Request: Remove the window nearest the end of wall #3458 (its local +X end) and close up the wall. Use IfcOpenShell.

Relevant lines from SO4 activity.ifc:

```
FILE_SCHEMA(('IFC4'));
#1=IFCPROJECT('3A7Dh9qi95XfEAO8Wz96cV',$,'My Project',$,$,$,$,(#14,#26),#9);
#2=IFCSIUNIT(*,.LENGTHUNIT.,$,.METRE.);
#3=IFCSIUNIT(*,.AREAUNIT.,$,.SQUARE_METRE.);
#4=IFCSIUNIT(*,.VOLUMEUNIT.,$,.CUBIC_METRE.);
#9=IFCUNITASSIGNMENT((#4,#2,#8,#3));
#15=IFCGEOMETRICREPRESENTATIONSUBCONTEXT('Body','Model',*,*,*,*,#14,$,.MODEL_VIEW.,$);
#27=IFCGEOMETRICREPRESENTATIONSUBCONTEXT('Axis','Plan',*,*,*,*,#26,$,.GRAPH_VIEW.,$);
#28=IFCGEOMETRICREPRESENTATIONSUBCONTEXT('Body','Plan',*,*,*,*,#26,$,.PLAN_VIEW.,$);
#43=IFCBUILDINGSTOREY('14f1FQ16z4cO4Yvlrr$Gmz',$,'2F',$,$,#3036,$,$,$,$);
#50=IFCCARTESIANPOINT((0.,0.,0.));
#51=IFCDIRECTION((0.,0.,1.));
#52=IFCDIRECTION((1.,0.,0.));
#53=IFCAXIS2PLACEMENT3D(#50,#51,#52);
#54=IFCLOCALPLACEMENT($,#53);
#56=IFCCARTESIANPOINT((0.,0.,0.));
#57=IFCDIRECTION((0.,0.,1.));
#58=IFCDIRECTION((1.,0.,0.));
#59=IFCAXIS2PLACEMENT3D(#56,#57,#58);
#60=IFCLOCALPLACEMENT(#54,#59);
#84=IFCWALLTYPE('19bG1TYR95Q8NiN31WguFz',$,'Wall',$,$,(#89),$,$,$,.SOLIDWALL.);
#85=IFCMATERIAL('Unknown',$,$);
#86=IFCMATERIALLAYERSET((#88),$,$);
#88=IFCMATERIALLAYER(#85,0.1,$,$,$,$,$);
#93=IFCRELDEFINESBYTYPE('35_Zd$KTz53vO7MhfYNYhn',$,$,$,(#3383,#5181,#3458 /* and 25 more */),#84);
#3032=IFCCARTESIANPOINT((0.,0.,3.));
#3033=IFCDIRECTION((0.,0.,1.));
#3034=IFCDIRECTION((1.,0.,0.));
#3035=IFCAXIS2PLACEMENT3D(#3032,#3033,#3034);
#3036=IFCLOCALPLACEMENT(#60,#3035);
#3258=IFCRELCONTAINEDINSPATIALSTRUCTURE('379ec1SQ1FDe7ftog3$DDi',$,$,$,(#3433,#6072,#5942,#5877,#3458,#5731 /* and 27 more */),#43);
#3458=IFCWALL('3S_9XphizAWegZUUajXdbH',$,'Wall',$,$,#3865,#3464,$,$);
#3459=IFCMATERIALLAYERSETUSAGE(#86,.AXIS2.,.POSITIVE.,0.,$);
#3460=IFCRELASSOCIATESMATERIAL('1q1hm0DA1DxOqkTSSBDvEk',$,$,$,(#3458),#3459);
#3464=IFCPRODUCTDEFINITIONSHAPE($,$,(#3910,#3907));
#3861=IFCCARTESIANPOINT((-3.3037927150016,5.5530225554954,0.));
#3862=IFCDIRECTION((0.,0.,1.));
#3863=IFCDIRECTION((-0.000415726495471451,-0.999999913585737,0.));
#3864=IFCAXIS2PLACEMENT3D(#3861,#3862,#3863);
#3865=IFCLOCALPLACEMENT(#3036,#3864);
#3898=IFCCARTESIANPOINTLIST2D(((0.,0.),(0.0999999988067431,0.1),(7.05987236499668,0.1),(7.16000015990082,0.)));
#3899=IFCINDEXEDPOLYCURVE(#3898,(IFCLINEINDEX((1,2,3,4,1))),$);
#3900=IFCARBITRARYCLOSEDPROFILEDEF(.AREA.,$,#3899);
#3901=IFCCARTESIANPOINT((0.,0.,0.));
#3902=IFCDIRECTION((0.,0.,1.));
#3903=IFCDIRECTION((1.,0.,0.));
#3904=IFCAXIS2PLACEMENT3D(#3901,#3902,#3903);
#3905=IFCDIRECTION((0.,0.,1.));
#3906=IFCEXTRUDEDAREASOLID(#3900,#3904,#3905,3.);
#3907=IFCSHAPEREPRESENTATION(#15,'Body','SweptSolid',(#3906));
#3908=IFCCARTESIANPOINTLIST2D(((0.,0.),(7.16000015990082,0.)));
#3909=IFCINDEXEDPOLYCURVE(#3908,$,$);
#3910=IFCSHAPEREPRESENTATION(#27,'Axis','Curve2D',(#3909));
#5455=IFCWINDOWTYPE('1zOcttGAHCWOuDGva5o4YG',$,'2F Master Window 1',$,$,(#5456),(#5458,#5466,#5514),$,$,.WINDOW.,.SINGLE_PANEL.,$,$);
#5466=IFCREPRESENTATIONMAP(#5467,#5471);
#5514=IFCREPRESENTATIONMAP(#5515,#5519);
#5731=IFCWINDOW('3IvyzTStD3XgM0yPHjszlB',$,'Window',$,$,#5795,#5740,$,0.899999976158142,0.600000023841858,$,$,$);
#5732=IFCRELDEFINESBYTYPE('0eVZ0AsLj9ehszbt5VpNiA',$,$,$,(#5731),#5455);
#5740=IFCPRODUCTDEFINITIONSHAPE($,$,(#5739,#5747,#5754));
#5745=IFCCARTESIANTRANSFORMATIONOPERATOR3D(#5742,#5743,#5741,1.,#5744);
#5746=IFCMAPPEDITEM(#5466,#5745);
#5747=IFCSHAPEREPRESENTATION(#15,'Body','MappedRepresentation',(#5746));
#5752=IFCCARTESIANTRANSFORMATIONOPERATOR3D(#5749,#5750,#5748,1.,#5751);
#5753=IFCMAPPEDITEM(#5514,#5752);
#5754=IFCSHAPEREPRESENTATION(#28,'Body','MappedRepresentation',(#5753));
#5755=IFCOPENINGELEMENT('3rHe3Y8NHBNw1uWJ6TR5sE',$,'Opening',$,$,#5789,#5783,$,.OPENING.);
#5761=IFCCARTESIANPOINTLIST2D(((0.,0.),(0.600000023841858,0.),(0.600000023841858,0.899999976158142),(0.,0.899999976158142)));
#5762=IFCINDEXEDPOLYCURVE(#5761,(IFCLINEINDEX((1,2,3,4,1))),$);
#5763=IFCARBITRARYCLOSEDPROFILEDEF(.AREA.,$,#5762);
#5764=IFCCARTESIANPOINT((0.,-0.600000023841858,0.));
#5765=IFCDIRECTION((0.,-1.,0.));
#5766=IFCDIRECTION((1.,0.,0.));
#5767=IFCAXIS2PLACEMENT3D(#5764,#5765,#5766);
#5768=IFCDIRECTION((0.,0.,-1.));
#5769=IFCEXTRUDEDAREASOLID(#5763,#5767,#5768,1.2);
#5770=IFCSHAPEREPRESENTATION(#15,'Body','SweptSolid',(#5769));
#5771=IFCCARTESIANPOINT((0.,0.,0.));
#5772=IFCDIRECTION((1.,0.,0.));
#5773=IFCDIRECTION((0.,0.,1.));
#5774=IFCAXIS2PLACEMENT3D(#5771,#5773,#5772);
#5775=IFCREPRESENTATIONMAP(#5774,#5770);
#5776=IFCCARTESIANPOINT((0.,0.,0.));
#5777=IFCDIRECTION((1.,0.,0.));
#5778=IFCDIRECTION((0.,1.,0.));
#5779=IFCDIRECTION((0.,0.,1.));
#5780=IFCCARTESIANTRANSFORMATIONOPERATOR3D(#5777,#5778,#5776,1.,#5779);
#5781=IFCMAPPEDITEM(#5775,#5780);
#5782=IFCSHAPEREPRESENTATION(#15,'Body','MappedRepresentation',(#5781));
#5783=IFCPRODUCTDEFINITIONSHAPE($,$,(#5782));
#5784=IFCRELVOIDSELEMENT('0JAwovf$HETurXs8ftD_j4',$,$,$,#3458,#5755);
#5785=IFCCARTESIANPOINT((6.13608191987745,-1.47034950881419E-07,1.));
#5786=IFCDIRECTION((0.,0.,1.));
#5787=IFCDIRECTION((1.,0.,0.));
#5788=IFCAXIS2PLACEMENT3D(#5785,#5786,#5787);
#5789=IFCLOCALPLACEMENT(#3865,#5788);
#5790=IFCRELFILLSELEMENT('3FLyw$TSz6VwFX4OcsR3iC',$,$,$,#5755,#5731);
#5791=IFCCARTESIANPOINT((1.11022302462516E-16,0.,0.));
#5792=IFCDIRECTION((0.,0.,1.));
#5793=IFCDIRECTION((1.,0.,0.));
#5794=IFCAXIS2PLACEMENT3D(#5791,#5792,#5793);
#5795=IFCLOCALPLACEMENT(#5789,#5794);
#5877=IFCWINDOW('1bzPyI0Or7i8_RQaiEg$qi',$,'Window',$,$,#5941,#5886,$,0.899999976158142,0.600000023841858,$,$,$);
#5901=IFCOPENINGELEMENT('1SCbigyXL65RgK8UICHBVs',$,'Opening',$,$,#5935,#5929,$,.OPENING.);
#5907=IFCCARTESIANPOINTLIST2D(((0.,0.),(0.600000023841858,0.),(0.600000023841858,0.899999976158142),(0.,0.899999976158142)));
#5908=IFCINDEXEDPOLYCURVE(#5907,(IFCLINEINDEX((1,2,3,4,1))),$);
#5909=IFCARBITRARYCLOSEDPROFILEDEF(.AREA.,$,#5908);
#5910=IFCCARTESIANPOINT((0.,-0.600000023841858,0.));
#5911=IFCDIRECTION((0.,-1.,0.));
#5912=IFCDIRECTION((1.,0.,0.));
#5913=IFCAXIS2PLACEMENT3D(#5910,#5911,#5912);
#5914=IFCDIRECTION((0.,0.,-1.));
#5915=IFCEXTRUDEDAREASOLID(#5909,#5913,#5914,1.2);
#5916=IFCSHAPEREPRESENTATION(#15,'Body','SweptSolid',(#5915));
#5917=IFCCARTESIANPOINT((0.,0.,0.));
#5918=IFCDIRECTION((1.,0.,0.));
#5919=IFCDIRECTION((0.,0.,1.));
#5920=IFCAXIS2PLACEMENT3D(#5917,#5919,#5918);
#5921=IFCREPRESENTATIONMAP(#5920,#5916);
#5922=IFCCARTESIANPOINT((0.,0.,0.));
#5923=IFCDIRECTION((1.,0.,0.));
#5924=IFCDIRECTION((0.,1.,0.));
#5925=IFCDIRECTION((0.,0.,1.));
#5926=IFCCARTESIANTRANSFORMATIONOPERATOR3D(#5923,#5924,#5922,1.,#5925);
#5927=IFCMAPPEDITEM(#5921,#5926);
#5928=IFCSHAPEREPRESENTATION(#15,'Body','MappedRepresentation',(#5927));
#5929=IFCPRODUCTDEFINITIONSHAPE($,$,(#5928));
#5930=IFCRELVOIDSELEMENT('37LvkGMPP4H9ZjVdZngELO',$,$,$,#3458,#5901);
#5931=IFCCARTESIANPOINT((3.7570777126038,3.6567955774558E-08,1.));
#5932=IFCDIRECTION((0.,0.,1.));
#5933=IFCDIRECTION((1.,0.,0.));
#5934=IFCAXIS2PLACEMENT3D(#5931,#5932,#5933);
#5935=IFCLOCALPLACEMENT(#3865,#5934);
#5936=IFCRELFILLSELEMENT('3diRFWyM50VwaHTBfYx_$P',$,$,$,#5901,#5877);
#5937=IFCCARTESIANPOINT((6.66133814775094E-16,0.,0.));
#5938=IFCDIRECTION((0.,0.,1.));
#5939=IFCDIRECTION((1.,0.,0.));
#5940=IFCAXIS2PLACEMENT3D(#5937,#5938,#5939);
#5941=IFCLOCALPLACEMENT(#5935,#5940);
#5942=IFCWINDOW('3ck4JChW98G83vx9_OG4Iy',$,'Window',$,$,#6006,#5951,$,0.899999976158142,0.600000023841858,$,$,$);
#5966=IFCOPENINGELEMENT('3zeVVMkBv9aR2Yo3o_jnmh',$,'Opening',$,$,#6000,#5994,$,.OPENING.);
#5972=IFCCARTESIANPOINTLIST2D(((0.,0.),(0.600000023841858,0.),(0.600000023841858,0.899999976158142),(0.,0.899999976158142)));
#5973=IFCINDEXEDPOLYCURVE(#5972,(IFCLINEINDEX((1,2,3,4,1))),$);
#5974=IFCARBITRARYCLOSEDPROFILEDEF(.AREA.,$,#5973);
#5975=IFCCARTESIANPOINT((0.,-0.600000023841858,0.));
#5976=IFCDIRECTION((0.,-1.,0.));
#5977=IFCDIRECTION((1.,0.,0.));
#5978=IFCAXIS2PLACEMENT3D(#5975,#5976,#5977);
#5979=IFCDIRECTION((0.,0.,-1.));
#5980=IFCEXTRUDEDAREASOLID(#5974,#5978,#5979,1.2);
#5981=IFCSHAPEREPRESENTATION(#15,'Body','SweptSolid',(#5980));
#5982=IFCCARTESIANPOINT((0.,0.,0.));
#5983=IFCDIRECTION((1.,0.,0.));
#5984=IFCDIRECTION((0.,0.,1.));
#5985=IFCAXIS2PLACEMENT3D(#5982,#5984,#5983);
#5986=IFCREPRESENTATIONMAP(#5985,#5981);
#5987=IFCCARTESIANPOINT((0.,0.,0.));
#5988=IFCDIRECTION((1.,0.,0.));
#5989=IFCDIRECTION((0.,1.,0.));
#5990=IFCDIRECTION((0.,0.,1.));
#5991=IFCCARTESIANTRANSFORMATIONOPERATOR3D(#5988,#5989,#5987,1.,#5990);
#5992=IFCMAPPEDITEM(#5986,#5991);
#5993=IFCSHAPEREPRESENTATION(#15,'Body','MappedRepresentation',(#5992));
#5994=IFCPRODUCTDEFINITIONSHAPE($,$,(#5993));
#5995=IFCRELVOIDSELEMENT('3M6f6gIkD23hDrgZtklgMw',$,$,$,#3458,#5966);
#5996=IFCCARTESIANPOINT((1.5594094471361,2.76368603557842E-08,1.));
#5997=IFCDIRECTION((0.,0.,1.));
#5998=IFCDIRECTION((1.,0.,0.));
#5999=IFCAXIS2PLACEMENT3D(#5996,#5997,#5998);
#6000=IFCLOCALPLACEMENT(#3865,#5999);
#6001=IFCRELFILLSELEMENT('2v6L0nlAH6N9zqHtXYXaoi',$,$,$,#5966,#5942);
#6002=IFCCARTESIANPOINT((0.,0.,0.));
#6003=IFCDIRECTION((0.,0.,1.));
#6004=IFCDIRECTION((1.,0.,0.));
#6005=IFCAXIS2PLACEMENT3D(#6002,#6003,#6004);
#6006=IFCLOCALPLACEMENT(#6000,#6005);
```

```python
import ifcopenshell
import ifcopenshell.api.feature
import ifcopenshell.api.root
import ifcopenshell.geom
import ifcopenshell.util.shape

model = ifcopenshell.open("SO4 activity.ifc")
settings = ifcopenshell.geom.settings()


def volume(element):
    """Net volume in cubic metres, openings subtracted."""
    shape = ifcopenshell.geom.create_shape(settings, element)
    return ifcopenshell.util.shape.get_volume(shape.geometry)


window = model.by_guid("3IvyzTStD3XgM0yPHjszlB")
opening = window.FillsVoids[0].RelatingOpeningElement
wall = opening.VoidsElements[0].RelatingBuildingElement
before = volume(wall)

ifcopenshell.api.root.remove_product(model, product=window)
ifcopenshell.api.feature.remove_feature(model, feature=opening)

after = volume(wall)

print(f"wall volume {before:.3f} -> {after:.3f} m3")

model.write("SO4 activity_v2.ifc")
```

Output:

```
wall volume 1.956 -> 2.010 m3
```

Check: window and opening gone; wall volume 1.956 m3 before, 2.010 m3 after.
